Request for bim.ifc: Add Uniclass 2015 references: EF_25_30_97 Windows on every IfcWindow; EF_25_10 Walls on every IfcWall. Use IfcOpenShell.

First a look at what the model holds.

```python
import ifcopenshell

model = ifcopenshell.open("bim.ifc")
print(model.schema)
print("classifications:", [c.Name for c in model.by_type("IfcClassification")])
for ifc_class in ("IfcDoor", "IfcRoof", "IfcStair", "IfcWall", "IfcWindow"):
    print(ifc_class, len(model.by_type(ifc_class)))
```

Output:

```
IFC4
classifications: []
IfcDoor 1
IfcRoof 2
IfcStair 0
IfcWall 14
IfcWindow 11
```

```python
import ifcopenshell
import ifcopenshell.api.classification

model = ifcopenshell.open("bim.ifc")

system = ifcopenshell.api.classification.add_classification(model, classification="Uniclass 2015")

codes = {
    "IfcWindow": ("EF_25_30_97", "Windows"),
    "IfcWall": ("EF_25_10", "Walls"),
}
for ifc_class, (code, name) in codes.items():
    products = model.by_type(ifc_class)
    ifcopenshell.api.classification.add_reference(
        model, products=products, classification=system, identification=code, name=name
    )
    print(code, len(products))

model.write("bim_rev.ifc")
```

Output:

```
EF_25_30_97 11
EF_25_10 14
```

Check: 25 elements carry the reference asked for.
